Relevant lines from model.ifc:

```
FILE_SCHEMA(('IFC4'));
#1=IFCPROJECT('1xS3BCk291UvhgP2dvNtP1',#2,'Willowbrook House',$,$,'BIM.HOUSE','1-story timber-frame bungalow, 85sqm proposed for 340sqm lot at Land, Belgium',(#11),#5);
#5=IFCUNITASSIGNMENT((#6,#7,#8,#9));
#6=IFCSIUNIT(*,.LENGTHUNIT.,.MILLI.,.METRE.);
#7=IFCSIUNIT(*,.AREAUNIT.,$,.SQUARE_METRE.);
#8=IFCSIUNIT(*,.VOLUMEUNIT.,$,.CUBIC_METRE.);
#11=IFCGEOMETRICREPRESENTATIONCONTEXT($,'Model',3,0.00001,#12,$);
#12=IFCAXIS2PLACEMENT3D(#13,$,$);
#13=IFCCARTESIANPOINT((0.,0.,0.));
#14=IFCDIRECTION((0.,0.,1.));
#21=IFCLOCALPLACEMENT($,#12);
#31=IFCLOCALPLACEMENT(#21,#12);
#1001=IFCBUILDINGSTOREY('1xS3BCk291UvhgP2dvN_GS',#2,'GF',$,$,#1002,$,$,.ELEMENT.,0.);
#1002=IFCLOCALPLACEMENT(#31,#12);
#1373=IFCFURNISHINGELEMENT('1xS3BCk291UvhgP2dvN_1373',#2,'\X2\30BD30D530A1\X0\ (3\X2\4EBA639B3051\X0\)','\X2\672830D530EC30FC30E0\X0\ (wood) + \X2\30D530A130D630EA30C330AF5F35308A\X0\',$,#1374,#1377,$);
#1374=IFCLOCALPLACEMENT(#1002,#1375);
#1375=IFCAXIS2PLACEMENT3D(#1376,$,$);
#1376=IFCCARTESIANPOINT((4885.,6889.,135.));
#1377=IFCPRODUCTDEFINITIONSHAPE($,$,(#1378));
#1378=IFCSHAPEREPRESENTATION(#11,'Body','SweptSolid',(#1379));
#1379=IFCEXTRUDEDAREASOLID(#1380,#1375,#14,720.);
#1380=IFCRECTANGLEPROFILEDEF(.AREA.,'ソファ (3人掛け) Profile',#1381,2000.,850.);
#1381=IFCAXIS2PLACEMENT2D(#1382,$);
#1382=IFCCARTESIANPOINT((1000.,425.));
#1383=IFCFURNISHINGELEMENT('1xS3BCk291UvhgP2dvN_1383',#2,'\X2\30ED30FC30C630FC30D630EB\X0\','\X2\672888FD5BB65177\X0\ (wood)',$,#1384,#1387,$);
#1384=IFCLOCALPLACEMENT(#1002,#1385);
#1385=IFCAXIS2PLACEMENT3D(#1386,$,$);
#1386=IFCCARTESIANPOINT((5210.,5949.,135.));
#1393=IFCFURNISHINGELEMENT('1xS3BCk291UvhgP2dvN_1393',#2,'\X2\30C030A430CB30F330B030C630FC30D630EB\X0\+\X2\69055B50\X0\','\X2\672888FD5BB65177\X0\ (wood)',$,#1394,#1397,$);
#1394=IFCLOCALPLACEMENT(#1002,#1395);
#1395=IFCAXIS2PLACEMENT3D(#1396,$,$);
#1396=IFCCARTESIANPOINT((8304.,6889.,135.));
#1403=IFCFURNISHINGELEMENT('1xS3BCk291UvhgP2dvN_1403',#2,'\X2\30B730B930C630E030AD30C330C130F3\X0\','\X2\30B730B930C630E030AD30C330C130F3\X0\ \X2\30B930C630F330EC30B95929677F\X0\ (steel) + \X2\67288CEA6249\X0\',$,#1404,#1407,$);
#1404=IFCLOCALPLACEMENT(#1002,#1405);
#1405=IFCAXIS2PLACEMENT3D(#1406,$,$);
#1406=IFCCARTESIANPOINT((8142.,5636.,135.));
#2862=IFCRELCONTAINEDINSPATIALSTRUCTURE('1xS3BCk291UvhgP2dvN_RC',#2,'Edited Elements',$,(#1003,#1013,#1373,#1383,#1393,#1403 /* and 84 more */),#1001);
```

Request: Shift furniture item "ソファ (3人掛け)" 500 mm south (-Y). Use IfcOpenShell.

```python
import ifcopenshell
import ifcopenshell.api.geometry
import ifcopenshell.util.placement
import ifcopenshell.util.unit

model = ifcopenshell.open("model.ifc")
unit_scale = ifcopenshell.util.unit.calculate_unit_scale(model)

item = model.by_id(1373)
matrix = ifcopenshell.util.placement.get_local_placement(item.ObjectPlacement)
matrix[1, 3] -= 0.5 / unit_scale
ifcopenshell.api.geometry.edit_object_placement(model, product=item, matrix=matrix, is_si=False)

print(ifcopenshell.util.placement.get_local_placement(item.ObjectPlacement).round(3) + 0.0)

model.write("model_updated.ifc")
```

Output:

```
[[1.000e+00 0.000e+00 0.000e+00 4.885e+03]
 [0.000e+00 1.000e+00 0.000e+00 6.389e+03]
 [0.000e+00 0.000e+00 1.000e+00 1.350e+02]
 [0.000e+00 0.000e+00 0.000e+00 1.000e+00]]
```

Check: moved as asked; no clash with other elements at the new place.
